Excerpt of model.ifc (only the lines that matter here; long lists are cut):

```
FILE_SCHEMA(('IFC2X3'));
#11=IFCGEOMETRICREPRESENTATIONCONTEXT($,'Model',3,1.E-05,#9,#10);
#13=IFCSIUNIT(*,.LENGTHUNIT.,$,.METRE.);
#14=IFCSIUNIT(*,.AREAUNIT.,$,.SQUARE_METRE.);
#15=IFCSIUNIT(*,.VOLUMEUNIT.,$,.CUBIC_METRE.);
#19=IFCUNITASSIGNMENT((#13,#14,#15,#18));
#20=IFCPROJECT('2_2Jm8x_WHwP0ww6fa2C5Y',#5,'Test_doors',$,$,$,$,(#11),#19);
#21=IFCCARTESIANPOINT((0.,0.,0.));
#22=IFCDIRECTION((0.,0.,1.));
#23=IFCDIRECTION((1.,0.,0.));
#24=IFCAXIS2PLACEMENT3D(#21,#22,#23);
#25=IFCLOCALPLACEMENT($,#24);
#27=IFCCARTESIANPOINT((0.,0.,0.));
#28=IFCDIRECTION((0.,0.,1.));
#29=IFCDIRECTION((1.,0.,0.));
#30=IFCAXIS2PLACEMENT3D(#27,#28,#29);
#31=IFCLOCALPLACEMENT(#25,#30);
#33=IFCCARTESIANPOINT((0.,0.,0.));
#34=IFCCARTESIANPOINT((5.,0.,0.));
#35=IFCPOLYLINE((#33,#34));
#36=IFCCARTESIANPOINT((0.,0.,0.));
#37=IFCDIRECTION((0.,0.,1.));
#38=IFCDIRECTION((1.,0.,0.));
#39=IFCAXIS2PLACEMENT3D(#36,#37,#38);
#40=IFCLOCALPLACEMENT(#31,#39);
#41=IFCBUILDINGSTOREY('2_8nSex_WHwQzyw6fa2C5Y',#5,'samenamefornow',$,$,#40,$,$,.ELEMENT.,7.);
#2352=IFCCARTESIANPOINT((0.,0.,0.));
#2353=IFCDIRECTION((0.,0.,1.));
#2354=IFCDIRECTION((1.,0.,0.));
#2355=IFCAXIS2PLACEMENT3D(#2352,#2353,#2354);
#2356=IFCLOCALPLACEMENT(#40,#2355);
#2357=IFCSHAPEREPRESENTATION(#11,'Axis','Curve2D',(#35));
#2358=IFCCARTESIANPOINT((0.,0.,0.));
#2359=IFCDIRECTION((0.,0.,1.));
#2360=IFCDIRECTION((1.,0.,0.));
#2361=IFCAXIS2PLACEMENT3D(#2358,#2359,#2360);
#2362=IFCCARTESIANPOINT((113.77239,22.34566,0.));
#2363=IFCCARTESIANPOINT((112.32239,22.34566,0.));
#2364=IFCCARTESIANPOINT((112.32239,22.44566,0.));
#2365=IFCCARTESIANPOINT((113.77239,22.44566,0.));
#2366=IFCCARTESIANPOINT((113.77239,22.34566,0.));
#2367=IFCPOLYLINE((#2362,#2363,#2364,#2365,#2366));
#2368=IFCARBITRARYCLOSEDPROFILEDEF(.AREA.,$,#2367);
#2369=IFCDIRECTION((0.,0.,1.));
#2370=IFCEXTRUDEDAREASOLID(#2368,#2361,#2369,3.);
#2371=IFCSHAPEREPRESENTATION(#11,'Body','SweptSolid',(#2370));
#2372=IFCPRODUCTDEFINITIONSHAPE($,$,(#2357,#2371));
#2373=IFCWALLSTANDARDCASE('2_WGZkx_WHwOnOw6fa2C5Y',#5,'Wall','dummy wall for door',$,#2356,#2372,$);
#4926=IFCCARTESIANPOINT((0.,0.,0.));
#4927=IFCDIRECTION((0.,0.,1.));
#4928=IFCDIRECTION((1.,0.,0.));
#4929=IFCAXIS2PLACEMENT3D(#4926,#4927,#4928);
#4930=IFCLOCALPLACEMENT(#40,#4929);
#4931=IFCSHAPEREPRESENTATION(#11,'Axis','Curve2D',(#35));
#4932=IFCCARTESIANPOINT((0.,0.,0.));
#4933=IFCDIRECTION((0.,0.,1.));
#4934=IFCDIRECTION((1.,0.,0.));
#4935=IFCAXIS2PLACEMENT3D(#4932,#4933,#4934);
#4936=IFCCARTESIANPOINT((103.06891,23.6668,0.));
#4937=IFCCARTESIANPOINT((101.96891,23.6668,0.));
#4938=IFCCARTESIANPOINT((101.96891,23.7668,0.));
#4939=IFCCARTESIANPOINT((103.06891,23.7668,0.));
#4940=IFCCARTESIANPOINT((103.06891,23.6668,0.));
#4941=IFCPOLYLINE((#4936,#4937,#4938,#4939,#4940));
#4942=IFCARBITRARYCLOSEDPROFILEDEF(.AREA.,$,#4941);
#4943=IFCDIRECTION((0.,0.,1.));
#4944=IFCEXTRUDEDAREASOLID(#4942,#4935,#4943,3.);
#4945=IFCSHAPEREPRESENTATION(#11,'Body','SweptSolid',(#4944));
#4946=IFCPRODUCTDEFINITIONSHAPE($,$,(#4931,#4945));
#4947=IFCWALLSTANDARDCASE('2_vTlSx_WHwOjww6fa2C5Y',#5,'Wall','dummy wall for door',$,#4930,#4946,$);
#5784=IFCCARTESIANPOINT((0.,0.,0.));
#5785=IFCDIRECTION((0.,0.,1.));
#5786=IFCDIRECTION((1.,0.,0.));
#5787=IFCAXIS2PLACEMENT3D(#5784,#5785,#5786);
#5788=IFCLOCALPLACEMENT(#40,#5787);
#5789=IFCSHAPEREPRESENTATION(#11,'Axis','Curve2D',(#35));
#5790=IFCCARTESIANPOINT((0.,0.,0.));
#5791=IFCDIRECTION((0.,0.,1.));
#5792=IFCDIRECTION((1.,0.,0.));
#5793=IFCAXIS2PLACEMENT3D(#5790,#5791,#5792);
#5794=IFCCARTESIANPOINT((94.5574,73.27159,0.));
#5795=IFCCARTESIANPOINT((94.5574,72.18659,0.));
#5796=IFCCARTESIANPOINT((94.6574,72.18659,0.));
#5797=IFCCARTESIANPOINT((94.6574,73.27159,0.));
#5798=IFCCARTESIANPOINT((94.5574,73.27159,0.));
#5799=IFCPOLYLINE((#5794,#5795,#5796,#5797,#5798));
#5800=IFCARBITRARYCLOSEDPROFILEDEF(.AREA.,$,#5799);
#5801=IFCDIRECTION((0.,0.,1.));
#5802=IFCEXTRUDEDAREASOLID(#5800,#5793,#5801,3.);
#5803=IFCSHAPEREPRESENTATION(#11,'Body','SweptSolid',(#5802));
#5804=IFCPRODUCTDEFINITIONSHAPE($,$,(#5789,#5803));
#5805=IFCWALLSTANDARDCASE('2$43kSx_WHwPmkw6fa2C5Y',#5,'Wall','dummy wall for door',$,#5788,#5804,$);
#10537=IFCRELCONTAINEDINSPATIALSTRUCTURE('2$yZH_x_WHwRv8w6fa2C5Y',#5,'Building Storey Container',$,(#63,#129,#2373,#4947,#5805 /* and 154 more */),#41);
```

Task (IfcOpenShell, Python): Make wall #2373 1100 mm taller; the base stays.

```python
import ifcopenshell
import ifcopenshell.geom
import ifcopenshell.util.shape

model = ifcopenshell.open("model.ifc")
settings = ifcopenshell.geom.settings()


def volume(element):
    """Net volume in cubic metres, openings subtracted."""
    shape = ifcopenshell.geom.create_shape(settings, element)
    return ifcopenshell.util.shape.get_volume(shape.geometry)


wall = model.by_guid("2_WGZkx_WHwOnOw6fa2C5Y")
before = volume(wall)

body = next(r for r in wall.Representation.Representations if r.RepresentationIdentifier == "Body")
solid = body.Items[0]
old_height = solid.Depth
solid.Depth += 1.1
after = volume(wall)

print(f"height {old_height:g} -> {solid.Depth:g}, volume {before:.3f} -> {after:.3f} m3")

model.write("model_updated.ifc")
```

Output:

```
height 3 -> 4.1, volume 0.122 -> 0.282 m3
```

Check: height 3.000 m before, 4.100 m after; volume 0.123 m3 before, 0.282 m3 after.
